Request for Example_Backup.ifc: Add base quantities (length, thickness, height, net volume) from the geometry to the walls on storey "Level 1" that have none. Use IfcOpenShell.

First a look at what the model holds.

```python
import ifcopenshell
import ifcopenshell.util.element
import ifcopenshell.util.unit

model = ifcopenshell.open("Example_Backup.ifc")
print(model.schema)
for unit_type in ("LENGTHUNIT", "AREAUNIT", "VOLUMEUNIT"):
    print(unit_type, ifcopenshell.util.unit.calculate_unit_scale(model, unit_type))
storey = next(s for s in model.by_type("IfcBuildingStorey") if s.Name == "Level 1")
walls = [e for e in ifcopenshell.util.element.get_decomposition(storey) if e.is_a("IfcWall")]
for e in sorted(walls, key=lambda e: e.id()):
    print(e.id(), e.is_a(), e.Name, list(ifcopenshell.util.element.get_psets(e, qtos_only=True)), sep=" | ")
```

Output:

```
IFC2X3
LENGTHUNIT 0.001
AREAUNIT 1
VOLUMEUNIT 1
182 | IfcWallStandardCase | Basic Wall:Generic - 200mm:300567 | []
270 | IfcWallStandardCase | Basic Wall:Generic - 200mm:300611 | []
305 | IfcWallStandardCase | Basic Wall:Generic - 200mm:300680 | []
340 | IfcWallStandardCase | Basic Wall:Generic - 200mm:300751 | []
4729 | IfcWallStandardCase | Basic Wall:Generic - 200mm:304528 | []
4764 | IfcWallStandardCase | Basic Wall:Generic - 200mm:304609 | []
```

```python
import ifcopenshell
import ifcopenshell.api.pset
import ifcopenshell.geom
import ifcopenshell.util.element
import ifcopenshell.util.shape
import ifcopenshell.util.unit

model = ifcopenshell.open("Example_Backup.ifc")
unit_scale = ifcopenshell.util.unit.calculate_unit_scale(model)
volume_scale = ifcopenshell.util.unit.calculate_unit_scale(model, "VOLUMEUNIT")
settings = ifcopenshell.geom.settings()

storey = next(s for s in model.by_type("IfcBuildingStorey") if s.Name == "Level 1")
walls = [e for e in ifcopenshell.util.element.get_decomposition(storey) if e.is_a("IfcWall")]

for e in sorted(walls, key=lambda e: e.id()):
    if ifcopenshell.util.element.get_psets(e, qtos_only=True, should_inherit=False):
        continue
    # Geometry comes back in metres, in the element's own axes.
    shape = ifcopenshell.geom.create_shape(settings, e)
    values = {
        "Length": ifcopenshell.util.shape.get_x(shape.geometry) / unit_scale,
        "Width": ifcopenshell.util.shape.get_y(shape.geometry) / unit_scale,
        "Height": ifcopenshell.util.shape.get_z(shape.geometry) / unit_scale,
        "NetVolume": ifcopenshell.util.shape.get_volume(shape.geometry) / volume_scale,
    }
    qto = ifcopenshell.api.pset.add_qto(model, product=e, name="BaseQuantities")
    ifcopenshell.api.pset.edit_qto(model, qto=qto, properties=values)
    print(e.id(), {k: round(v, 3) for k, v in values.items()})

model.write("Example_Backup_updated.ifc")
```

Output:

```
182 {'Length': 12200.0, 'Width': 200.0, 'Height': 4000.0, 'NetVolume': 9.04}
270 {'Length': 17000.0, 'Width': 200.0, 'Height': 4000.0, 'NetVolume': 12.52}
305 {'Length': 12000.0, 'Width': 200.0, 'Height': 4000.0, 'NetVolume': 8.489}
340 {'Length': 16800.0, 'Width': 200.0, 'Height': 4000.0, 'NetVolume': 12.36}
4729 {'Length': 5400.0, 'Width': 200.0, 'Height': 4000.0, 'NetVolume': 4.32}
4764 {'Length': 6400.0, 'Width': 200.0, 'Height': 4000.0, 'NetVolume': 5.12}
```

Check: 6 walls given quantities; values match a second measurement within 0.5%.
